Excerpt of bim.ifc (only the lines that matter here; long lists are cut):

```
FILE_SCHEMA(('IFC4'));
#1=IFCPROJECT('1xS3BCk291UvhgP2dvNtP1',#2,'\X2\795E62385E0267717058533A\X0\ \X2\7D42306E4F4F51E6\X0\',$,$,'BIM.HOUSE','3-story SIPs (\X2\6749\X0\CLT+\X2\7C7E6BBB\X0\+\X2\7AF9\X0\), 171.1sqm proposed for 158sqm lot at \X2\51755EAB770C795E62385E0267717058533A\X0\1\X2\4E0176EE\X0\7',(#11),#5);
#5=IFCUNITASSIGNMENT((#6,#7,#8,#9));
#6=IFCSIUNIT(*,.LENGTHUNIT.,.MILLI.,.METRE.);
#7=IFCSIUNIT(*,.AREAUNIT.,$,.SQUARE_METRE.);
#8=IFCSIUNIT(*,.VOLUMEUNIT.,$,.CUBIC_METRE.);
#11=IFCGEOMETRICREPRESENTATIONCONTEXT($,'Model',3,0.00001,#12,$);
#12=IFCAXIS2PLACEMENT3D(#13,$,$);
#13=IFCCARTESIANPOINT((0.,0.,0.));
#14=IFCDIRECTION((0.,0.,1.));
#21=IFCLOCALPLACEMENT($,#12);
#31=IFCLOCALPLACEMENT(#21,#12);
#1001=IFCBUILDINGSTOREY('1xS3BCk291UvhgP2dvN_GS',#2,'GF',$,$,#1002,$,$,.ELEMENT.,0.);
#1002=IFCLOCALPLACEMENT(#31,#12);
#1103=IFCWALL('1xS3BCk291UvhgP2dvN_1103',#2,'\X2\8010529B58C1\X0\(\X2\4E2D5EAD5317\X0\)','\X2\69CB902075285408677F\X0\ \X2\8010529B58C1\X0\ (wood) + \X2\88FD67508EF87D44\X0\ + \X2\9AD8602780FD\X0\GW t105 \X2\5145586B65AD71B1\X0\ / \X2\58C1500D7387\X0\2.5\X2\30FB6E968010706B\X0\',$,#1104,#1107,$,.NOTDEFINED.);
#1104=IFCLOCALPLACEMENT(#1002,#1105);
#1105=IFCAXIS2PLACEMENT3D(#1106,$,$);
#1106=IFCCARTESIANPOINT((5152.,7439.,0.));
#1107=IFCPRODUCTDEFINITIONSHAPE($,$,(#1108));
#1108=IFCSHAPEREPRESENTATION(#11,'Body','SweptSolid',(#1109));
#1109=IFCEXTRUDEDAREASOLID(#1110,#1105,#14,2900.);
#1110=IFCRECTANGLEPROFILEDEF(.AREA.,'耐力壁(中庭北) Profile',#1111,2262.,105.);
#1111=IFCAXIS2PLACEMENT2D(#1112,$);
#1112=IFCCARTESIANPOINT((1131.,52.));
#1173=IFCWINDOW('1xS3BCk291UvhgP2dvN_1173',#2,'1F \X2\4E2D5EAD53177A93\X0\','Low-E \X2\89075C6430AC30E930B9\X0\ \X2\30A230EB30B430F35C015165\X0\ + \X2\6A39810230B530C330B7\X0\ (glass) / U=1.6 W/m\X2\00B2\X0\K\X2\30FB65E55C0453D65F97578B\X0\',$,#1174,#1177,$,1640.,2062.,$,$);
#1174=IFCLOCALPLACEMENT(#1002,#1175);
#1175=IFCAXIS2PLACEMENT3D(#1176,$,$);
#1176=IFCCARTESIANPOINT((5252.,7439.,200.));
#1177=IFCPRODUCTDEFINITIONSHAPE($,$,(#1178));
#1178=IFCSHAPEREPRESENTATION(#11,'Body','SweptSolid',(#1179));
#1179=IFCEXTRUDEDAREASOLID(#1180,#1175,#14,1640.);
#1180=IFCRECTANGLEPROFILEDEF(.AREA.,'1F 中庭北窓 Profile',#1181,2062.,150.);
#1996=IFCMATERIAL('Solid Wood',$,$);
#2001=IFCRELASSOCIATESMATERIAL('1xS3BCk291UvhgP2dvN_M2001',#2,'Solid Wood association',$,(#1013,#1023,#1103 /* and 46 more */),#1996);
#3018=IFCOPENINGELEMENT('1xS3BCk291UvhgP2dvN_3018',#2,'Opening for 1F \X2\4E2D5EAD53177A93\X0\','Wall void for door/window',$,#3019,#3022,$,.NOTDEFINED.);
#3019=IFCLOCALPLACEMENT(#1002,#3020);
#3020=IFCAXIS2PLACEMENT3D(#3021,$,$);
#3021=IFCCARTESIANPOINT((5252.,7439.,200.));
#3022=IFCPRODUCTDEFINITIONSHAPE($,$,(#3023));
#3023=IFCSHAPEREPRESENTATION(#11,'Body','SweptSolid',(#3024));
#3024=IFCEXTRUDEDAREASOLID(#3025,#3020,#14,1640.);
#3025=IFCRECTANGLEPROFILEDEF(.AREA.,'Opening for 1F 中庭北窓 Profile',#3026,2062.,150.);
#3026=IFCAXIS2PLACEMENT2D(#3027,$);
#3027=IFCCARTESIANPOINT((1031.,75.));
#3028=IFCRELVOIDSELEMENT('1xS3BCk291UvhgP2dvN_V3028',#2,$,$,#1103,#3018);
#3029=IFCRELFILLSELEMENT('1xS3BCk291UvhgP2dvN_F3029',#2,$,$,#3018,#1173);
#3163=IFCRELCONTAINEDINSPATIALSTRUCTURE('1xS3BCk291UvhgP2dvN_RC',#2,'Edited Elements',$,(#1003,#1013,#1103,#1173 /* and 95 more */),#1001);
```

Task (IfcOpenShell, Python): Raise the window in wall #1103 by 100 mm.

```python
import numpy as np
import ifcopenshell
import ifcopenshell.api.geometry
import ifcopenshell.util.placement
import ifcopenshell.util.unit

model = ifcopenshell.open("bim.ifc")
unit_scale = ifcopenshell.util.unit.calculate_unit_scale(model)

window = model.by_id(1173)
opening = window.FillsVoids[0].RelatingOpeningElement
dz = 0.1 / unit_scale

shift = np.array([0.0, 0.0, dz])
# The window is not placed relative to its opening, so move both.
for product in (opening, window):
    matrix = ifcopenshell.util.placement.get_local_placement(product.ObjectPlacement)
    matrix[:3, 3] += shift
    ifcopenshell.api.geometry.edit_object_placement(model, product=product, matrix=matrix, is_si=False)

print(f"moved by {dz * unit_scale:+.3f} m")

model.write("bim_updated.ifc")
```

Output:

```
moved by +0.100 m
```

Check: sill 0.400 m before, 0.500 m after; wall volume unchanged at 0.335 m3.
